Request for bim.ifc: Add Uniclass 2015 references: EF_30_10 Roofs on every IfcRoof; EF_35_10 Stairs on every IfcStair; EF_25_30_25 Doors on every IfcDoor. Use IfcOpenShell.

First a look at what the model holds.

```python
import ifcopenshell

model = ifcopenshell.open("bim.ifc")
print(model.schema)
print("classifications:", [c.Name for c in model.by_type("IfcClassification")])
for ifc_class in ("IfcDoor", "IfcRoof", "IfcStair", "IfcWall", "IfcWindow"):
    print(ifc_class, len(model.by_type(ifc_class)))
```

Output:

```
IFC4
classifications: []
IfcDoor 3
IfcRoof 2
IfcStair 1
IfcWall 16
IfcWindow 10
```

```python
import ifcopenshell
import ifcopenshell.api.classification

model = ifcopenshell.open("bim.ifc")

system = ifcopenshell.api.classification.add_classification(model, classification="Uniclass 2015")

codes = {
    "IfcRoof": ("EF_30_10", "Roofs"),
    "IfcStair": ("EF_35_10", "Stairs"),
    "IfcDoor": ("EF_25_30_25", "Doors"),
}
for ifc_class, (code, name) in codes.items():
    products = model.by_type(ifc_class)
    ifcopenshell.api.classification.add_reference(
        model, products=products, classification=system, identification=code, name=name
    )
    print(code, len(products))

model.write("bim-out.ifc")
```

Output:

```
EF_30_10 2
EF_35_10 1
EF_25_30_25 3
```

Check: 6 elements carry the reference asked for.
